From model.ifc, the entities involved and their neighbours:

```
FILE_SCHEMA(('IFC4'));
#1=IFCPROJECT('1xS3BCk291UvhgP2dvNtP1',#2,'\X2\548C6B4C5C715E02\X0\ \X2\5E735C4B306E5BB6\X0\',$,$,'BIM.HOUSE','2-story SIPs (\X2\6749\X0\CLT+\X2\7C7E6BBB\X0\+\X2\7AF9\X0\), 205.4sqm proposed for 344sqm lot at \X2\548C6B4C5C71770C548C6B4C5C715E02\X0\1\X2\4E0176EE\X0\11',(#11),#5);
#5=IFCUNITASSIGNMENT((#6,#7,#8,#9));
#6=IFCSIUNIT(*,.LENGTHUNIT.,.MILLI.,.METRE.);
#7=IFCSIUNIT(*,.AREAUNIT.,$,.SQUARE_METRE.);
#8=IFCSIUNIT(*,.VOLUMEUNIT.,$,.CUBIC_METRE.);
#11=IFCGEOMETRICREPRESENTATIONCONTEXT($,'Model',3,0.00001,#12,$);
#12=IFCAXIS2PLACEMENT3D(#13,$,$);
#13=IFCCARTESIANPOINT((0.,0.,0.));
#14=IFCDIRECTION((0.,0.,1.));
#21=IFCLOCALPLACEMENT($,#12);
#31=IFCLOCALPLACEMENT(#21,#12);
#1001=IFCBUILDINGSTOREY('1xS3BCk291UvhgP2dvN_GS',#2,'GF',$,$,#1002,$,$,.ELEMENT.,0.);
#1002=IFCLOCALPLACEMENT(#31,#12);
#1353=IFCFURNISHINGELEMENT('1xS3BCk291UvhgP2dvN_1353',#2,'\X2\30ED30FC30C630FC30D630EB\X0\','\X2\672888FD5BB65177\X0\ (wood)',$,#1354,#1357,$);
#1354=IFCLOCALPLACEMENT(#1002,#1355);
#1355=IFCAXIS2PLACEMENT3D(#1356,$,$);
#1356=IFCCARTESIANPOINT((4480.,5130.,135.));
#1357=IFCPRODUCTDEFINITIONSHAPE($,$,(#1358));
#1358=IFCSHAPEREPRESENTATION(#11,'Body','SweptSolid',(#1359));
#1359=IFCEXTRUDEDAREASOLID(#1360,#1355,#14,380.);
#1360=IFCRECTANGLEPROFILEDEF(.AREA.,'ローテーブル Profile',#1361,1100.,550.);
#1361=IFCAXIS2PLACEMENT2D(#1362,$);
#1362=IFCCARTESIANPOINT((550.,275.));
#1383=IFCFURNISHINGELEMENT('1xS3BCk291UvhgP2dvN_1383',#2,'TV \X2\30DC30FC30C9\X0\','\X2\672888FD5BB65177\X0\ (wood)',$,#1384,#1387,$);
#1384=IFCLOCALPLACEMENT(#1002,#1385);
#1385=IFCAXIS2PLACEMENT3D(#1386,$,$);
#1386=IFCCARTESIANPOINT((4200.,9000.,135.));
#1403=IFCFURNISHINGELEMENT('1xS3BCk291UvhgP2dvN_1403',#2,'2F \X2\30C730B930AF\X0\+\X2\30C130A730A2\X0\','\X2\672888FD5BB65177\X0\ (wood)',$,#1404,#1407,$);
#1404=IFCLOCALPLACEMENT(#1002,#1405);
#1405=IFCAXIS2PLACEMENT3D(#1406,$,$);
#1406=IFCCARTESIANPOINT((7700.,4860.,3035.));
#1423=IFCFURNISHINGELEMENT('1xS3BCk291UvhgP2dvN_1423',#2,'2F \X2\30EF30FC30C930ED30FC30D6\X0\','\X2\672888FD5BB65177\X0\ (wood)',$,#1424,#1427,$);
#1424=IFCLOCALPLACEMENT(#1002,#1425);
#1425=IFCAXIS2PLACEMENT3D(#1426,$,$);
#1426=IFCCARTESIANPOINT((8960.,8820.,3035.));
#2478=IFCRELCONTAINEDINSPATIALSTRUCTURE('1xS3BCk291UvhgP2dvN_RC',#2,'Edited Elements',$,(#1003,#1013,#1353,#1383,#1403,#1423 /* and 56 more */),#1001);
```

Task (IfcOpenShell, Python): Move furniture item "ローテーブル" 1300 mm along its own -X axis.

```python
import ifcopenshell
import ifcopenshell.api.geometry
import ifcopenshell.util.placement
import ifcopenshell.util.unit

model = ifcopenshell.open("model.ifc")
unit_scale = ifcopenshell.util.unit.calculate_unit_scale(model)

item = model.by_guid("1xS3BCk291UvhgP2dvN_1353")
matrix = ifcopenshell.util.placement.get_local_placement(item.ObjectPlacement)
matrix[:3, 3] -= matrix[:3, 0] * 1.3 / unit_scale
ifcopenshell.api.geometry.edit_object_placement(model, product=item, matrix=matrix, is_si=False)

print(ifcopenshell.util.placement.get_local_placement(item.ObjectPlacement).round(3) + 0.0)

model.write("model-out.ifc")
```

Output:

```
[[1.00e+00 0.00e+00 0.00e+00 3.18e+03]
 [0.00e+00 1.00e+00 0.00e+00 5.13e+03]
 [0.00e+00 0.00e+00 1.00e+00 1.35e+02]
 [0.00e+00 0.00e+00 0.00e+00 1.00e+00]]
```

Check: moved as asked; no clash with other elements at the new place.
